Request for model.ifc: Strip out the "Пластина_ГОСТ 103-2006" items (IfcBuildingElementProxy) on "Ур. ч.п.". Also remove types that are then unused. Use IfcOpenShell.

First a look at what the model holds.

```python
import ifcopenshell
import ifcopenshell.util.element

model = ifcopenshell.open("model.ifc")
print(model.schema)
storey = next(s for s in model.by_type("IfcBuildingStorey") if s.Name == "Ур. ч.п.")
proxies = [e for e in ifcopenshell.util.element.get_decomposition(storey) if e.is_a("IfcBuildingElementProxy")]
seen = {}
for e in proxies:
    element_type = ifcopenshell.util.element.get_type(e)
    name = element_type.Name if element_type not in (None, e) else None
    seen[name] = seen.get(name, 0) + 1
for name, count in sorted(seen.items(), key=str):
    print(count, "x", name)
```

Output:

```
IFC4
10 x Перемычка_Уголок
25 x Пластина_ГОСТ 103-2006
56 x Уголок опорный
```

```python
import ifcopenshell
import ifcopenshell.api.root
import ifcopenshell.util.element

model = ifcopenshell.open("model.ifc")

storey = next(s for s in model.by_type("IfcBuildingStorey") if s.Name == "Ур. ч.п.")
proxies = [e for e in ifcopenshell.util.element.get_decomposition(storey) if e.is_a("IfcBuildingElementProxy")]
targets = [e for e in proxies if (t := ifcopenshell.util.element.get_type(e)) not in (None, e) and t.Name == "Пластина_ГОСТ 103-2006"]
types = {ifcopenshell.util.element.get_type(e) for e in targets} - {None, *targets}

for e in targets:
    ifcopenshell.api.root.remove_product(model, product=e)
print(len(targets), "removed")

unused = [t for t in types if not ifcopenshell.util.element.get_types(t)]
for t in unused:
    ifcopenshell.api.root.remove_product(model, product=t)
print(len(unused), "unused types removed")

model.write("model_rev.ifc")
```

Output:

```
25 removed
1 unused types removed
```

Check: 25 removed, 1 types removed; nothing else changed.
